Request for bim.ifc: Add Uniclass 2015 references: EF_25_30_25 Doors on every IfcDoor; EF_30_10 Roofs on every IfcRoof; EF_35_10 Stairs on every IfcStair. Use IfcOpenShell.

First a look at what the model holds.

```python
import ifcopenshell

model = ifcopenshell.open("bim.ifc")
print(model.schema)
print("classifications:", [c.Name for c in model.by_type("IfcClassification")])
for ifc_class in ("IfcDoor", "IfcRoof", "IfcStair", "IfcWall", "IfcWindow"):
    print(ifc_class, len(model.by_type(ifc_class)))
```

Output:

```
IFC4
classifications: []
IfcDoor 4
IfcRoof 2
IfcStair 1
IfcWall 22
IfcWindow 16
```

```python
import ifcopenshell
import ifcopenshell.api.classification

model = ifcopenshell.open("bim.ifc")

system = ifcopenshell.api.classification.add_classification(model, classification="Uniclass 2015")

codes = {
    "IfcDoor": ("EF_25_30_25", "Doors"),
    "IfcRoof": ("EF_30_10", "Roofs"),
    "IfcStair": ("EF_35_10", "Stairs"),
}
for ifc_class, (code, name) in codes.items():
    products = model.by_type(ifc_class)
    ifcopenshell.api.classification.add_reference(
        model, products=products, classification=system, identification=code, name=name
    )
    print(code, len(products))

model.write("bim-out.ifc")
```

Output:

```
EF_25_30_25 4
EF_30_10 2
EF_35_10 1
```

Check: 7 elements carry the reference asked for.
